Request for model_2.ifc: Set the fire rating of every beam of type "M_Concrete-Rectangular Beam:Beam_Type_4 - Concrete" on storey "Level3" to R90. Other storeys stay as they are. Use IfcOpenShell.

First a look at what the model holds.

```python
import ifcopenshell
import ifcopenshell.util.element

model = ifcopenshell.open("model_2.ifc")
print(model.schema)
storey = next(s for s in model.by_type("IfcBuildingStorey") if s.Name == "Level3")
beams = [e for e in ifcopenshell.util.element.get_decomposition(storey) if e.is_a("IfcBeam")]
seen = {}
for e in beams:
    element_type = ifcopenshell.util.element.get_type(e)
    key = (element_type.Name if element_type != e and element_type else None, ifcopenshell.util.element.get_pset(e, "Pset_BeamCommon", "FireRating"))
    seen[key] = seen.get(key, 0) + 1
for (name, value), count in sorted(seen.items(), key=str):
    print(count, "x", name, "|", value)
```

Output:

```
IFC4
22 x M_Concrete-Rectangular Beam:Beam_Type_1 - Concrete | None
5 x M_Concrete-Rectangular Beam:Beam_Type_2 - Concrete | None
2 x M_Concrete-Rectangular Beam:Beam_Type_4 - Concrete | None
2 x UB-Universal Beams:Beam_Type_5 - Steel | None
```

```python
import ifcopenshell
import ifcopenshell.api.pset
import ifcopenshell.util.element

model = ifcopenshell.open("model_2.ifc")

storey = next(s for s in model.by_type("IfcBuildingStorey") if s.Name == "Level3")
beams = [e for e in ifcopenshell.util.element.get_decomposition(storey) if e.is_a("IfcBeam")]

count = 0
for e in beams:
    element_type = ifcopenshell.util.element.get_type(e)
    if element_type in (None, e) or element_type.Name != "M_Concrete-Rectangular Beam:Beam_Type_4 - Concrete":
        continue
    # add_pset returns the element's existing set when there is one.
    pset = ifcopenshell.api.pset.add_pset(model, product=e, name="Pset_BeamCommon")
    ifcopenshell.api.pset.edit_pset(model, pset=pset, properties={"FireRating": "R90"})
    count += 1

print(count, "beams updated")

model.write("model_2_edited.ifc")
```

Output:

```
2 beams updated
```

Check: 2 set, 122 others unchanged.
